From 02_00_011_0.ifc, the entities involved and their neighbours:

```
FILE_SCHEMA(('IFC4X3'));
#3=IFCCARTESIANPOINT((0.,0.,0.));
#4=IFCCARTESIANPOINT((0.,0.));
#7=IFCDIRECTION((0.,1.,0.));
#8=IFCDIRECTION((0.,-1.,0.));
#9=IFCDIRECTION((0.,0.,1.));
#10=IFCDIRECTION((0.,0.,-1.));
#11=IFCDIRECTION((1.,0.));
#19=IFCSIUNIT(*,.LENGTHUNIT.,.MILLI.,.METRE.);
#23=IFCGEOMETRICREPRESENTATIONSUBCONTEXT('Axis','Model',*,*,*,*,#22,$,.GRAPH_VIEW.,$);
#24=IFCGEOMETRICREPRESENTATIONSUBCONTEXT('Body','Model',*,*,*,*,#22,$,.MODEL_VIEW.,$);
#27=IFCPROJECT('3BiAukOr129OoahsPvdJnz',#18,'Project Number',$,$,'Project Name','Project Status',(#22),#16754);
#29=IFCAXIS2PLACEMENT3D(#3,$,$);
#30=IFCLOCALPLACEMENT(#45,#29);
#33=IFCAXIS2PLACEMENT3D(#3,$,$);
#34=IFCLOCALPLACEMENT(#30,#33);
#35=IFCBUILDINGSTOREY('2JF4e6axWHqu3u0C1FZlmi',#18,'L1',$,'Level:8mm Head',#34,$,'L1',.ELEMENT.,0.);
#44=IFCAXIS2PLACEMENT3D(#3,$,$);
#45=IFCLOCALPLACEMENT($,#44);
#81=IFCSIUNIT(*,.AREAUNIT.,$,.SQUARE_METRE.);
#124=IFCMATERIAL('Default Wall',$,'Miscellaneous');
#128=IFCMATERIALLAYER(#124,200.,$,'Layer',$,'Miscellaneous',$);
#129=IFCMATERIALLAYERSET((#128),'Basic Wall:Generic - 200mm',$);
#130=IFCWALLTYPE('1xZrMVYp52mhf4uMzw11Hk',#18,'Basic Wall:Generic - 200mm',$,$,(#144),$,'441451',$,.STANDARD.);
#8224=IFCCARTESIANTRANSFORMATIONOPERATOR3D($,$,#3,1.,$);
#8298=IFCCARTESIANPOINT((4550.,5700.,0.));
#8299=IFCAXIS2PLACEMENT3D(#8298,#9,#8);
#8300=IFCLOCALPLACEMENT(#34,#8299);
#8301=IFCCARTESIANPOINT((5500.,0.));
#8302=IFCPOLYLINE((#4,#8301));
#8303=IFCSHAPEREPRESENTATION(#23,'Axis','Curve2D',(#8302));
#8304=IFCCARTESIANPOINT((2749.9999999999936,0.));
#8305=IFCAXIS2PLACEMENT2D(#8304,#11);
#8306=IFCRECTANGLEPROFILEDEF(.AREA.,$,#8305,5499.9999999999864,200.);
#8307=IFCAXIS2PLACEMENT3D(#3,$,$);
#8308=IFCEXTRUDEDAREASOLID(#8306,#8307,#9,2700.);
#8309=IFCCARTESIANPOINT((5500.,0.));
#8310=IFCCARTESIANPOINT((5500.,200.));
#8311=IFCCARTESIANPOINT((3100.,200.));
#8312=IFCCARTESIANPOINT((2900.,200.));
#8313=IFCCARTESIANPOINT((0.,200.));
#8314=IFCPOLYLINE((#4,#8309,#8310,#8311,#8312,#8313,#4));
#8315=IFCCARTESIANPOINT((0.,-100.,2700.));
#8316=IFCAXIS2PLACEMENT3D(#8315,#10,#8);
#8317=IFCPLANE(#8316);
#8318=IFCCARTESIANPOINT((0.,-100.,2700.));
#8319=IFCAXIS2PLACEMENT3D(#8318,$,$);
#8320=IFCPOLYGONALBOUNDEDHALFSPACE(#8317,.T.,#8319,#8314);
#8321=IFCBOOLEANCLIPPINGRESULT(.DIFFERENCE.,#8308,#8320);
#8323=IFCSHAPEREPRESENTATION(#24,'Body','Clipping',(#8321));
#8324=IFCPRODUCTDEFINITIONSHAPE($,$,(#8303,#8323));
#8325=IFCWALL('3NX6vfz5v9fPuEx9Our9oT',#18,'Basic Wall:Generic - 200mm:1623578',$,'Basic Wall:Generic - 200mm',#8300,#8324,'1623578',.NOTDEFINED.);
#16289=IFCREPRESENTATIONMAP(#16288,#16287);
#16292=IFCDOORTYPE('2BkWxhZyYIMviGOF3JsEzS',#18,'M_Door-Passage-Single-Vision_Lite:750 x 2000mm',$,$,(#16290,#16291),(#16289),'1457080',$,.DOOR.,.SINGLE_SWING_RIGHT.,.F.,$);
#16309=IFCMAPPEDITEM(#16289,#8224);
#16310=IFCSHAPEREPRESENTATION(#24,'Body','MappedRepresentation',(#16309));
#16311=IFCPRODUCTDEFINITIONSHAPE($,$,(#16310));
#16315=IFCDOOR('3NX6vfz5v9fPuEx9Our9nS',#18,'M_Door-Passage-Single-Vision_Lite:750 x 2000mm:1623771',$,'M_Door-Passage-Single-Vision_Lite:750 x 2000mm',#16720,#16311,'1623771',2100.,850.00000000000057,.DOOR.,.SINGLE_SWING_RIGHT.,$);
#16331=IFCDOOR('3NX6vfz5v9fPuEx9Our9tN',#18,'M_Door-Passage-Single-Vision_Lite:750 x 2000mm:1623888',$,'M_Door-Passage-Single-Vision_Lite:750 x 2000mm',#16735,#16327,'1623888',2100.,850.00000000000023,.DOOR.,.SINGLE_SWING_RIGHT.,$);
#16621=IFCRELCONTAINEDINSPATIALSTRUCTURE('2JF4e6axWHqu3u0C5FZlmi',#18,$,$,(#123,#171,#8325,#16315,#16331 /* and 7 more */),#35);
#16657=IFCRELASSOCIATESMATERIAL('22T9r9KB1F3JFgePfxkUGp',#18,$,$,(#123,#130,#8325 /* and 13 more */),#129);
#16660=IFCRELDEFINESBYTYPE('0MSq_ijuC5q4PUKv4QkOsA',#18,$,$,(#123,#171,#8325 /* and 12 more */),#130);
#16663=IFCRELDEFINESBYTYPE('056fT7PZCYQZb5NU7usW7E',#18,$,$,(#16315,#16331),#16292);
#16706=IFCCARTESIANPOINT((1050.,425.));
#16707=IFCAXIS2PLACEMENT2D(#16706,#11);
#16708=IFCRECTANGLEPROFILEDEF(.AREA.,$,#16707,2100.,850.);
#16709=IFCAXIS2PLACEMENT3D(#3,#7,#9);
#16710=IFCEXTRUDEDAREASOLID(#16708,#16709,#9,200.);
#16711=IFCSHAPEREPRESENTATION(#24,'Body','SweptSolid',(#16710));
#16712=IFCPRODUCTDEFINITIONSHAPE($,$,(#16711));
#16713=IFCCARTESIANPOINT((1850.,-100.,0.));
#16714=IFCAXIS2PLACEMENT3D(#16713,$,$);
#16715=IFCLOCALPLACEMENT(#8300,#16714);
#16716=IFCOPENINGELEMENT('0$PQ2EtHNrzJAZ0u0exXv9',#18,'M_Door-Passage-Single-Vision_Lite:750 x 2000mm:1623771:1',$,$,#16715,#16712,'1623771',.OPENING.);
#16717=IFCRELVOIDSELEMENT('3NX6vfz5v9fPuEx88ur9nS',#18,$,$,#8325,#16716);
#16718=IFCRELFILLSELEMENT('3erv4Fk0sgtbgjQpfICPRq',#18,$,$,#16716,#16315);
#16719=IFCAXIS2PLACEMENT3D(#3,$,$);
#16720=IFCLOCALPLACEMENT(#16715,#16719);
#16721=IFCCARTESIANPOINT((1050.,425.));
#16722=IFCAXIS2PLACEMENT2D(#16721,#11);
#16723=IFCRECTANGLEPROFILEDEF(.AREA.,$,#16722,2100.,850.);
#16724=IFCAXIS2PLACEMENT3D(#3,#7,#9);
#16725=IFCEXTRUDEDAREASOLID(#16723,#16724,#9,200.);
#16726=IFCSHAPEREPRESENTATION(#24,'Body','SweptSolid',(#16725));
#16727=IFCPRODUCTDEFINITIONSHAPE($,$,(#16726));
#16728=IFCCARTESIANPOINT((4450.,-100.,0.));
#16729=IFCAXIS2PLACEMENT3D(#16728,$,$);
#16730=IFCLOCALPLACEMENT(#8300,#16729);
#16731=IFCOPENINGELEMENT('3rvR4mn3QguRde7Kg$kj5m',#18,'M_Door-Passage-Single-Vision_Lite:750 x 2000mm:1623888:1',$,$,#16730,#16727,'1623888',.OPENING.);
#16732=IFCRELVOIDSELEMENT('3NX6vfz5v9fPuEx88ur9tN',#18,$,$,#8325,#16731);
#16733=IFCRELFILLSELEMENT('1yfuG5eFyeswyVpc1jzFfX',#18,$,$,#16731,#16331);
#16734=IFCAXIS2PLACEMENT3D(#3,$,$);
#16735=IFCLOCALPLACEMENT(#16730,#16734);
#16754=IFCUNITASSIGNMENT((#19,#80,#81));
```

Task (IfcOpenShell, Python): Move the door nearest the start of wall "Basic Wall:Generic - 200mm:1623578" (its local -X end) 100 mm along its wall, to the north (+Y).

```python
import ifcopenshell
import ifcopenshell.api.geometry
import ifcopenshell.util.placement
import ifcopenshell.util.unit

model = ifcopenshell.open("02_00_011_0.ifc")
unit_scale = ifcopenshell.util.unit.calculate_unit_scale(model)

door = model.by_guid("3NX6vfz5v9fPuEx9Our9nS")
opening = door.FillsVoids[0].RelatingOpeningElement
wall = opening.VoidsElements[0].RelatingBuildingElement

wall_matrix = ifcopenshell.util.placement.get_local_placement(wall.ObjectPlacement)
shift = wall_matrix[:3, 0] * -0.1 / unit_scale
before = ifcopenshell.util.placement.get_local_placement(door.ObjectPlacement)[:3, 3].copy()

# The door is placed relative to its opening, so it follows when the opening moves.
matrix = ifcopenshell.util.placement.get_local_placement(opening.ObjectPlacement)
matrix[:3, 3] += shift
ifcopenshell.api.geometry.edit_object_placement(
    model, product=opening, matrix=matrix, is_si=False, should_transform_children=True
)

after = ifcopenshell.util.placement.get_local_placement(door.ObjectPlacement)[:3, 3]
print("door moved by", (after - before).round(3) + 0.0)

model.write("02_00_011_0_edited.ifc")
```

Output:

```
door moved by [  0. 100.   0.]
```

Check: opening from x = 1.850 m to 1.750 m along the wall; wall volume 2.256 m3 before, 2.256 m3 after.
